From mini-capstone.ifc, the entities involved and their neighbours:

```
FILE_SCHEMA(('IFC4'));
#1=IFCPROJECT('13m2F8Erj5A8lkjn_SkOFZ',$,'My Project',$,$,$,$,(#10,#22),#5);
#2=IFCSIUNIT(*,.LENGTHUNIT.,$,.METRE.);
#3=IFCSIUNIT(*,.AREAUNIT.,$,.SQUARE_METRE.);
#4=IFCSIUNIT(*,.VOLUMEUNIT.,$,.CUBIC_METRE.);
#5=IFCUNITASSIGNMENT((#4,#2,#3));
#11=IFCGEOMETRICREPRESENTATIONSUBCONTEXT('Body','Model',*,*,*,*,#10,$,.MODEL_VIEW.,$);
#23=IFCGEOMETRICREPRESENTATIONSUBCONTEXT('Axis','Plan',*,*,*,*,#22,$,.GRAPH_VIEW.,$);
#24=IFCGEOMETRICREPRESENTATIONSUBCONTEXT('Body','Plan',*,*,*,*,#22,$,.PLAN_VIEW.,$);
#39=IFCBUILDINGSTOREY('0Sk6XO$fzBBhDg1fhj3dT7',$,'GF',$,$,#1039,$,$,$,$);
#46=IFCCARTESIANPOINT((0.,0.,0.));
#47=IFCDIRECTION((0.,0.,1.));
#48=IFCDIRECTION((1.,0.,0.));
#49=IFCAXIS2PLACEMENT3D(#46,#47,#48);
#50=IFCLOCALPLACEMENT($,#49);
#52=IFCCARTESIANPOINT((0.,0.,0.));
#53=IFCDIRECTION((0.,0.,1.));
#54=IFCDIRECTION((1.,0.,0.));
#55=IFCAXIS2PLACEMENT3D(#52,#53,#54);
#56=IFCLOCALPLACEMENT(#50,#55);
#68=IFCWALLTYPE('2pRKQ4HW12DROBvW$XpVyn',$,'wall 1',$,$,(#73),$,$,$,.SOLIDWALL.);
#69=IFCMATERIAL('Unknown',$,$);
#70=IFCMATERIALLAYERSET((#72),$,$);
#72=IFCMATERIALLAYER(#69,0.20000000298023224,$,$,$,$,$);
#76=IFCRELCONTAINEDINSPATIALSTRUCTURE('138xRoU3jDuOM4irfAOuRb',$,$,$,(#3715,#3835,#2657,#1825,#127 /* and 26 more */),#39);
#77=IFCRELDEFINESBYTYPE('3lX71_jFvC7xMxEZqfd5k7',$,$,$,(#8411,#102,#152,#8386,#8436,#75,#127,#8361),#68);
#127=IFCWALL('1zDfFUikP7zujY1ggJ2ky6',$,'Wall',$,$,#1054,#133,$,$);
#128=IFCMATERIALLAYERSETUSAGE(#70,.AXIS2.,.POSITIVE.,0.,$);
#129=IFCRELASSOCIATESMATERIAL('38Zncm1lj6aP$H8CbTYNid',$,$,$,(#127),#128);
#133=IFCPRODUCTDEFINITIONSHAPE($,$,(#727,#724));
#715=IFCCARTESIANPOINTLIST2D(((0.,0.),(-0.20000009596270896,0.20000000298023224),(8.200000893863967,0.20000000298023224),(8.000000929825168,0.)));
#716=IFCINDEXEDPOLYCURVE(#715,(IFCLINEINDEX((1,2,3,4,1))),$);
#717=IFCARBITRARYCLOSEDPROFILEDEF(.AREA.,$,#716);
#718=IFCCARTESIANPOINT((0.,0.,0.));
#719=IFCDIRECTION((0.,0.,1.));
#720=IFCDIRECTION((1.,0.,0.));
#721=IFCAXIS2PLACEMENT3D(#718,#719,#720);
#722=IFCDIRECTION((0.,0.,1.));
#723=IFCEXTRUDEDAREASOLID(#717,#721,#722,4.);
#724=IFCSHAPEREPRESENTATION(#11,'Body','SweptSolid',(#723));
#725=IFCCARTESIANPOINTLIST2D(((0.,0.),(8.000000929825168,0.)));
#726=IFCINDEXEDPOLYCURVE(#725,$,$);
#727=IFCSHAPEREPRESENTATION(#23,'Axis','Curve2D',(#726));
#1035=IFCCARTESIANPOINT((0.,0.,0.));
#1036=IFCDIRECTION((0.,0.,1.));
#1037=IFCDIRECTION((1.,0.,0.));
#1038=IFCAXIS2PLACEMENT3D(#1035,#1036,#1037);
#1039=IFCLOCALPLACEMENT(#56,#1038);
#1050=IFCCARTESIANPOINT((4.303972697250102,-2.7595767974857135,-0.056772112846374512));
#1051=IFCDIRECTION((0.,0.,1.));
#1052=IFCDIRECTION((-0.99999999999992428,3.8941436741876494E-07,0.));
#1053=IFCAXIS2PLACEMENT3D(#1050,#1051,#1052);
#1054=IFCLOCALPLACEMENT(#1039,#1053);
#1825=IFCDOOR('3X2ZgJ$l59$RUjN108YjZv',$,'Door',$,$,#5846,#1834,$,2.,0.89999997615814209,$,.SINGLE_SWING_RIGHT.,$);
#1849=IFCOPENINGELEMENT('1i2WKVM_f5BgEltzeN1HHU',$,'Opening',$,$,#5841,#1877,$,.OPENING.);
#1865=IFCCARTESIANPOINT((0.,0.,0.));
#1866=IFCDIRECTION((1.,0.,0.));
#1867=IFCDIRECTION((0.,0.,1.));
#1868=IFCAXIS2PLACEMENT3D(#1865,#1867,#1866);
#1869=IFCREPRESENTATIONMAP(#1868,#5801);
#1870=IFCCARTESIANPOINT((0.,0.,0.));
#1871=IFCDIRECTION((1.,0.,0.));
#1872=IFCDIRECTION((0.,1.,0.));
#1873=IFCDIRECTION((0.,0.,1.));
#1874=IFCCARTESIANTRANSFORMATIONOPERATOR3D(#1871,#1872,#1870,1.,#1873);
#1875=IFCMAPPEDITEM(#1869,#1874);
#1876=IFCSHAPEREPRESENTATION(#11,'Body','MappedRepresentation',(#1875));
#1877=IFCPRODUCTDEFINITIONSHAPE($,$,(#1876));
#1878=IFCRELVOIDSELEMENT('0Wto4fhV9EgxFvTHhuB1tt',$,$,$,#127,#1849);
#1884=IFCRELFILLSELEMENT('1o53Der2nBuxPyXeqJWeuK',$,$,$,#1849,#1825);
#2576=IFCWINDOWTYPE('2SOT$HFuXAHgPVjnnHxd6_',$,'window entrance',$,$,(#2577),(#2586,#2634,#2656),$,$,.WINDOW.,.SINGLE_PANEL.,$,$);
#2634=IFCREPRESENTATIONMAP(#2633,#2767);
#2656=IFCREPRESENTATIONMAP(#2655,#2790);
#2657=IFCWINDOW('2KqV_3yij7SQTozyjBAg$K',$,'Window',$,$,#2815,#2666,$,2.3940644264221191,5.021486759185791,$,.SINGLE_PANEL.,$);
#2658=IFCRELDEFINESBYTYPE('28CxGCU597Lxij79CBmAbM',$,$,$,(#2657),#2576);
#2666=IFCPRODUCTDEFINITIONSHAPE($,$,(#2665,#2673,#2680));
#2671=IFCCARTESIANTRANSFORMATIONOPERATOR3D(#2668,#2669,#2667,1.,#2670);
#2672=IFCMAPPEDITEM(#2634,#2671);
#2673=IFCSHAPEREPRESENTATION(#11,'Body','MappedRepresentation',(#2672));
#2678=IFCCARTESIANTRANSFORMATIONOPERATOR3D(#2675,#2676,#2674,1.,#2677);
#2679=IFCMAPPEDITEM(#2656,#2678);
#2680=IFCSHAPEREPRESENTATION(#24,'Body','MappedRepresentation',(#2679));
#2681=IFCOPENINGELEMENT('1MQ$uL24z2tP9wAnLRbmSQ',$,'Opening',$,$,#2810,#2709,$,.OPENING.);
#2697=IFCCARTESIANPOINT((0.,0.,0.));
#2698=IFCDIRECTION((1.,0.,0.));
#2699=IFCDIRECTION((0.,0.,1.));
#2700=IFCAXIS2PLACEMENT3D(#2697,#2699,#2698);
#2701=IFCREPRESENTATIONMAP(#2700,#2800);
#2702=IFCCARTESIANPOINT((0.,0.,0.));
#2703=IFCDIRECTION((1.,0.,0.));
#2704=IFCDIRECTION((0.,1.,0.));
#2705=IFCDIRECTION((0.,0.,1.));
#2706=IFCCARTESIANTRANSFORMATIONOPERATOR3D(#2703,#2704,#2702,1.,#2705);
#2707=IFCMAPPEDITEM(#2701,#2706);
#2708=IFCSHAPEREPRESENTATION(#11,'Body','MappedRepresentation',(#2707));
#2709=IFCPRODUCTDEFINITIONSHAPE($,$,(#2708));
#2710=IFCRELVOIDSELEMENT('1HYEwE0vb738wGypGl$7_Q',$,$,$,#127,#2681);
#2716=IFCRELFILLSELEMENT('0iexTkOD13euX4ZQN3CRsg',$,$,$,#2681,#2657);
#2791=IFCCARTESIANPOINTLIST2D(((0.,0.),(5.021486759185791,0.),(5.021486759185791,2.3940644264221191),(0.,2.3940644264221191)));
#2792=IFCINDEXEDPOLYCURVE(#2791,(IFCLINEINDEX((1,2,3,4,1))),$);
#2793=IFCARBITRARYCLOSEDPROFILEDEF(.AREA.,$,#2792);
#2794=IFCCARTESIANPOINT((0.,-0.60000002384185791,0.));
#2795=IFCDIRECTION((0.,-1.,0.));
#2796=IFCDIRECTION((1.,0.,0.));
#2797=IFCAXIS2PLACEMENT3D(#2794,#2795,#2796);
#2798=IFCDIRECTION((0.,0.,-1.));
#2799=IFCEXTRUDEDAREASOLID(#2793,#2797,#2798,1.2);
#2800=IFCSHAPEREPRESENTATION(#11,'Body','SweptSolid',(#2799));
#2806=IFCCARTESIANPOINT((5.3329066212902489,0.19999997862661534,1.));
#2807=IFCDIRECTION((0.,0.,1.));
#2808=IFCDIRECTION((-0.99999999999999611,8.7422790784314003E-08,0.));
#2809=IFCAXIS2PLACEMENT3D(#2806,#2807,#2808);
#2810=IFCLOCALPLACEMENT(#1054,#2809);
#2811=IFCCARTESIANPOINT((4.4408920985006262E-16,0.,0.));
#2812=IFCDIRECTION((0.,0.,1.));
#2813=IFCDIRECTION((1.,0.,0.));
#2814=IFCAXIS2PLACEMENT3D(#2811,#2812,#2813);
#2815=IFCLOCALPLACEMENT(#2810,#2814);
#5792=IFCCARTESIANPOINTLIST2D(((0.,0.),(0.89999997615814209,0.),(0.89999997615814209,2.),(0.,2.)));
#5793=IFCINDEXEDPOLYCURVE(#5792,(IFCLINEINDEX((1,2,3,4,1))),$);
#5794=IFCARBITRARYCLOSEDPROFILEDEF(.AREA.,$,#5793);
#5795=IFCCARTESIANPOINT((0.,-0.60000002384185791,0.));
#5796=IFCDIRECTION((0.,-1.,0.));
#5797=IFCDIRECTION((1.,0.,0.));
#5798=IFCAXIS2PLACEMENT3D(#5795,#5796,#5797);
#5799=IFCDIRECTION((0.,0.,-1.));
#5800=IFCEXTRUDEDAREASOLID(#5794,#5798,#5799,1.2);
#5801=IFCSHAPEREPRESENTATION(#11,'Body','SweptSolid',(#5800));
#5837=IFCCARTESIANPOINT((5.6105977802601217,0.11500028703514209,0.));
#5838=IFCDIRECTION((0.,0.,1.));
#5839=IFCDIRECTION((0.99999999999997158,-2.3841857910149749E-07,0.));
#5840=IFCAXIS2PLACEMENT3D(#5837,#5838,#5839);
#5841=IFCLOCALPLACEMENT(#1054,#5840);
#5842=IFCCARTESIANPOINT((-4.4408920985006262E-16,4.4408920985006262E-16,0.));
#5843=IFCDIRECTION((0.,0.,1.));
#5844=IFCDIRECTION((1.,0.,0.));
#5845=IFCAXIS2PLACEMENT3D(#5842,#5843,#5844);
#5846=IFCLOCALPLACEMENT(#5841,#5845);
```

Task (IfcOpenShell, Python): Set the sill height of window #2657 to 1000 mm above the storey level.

```python
import numpy as np
import ifcopenshell
import ifcopenshell.api.geometry
import ifcopenshell.geom
import ifcopenshell.util.element
import ifcopenshell.util.placement
import ifcopenshell.util.shape
import ifcopenshell.util.unit

model = ifcopenshell.open("mini-capstone.ifc")
unit_scale = ifcopenshell.util.unit.calculate_unit_scale(model)

window = model.by_id(2657)
opening = window.FillsVoids[0].RelatingOpeningElement
storey = ifcopenshell.util.element.get_container(window, ifc_class="IfcBuildingStorey")
level = ifcopenshell.util.placement.get_local_placement(storey.ObjectPlacement)[2, 3]

# The opening's origin need not be at the sill, so measure its lowest point.
shape = ifcopenshell.geom.create_shape(ifcopenshell.geom.settings(), opening)
bottom = ifcopenshell.util.shape.get_shape_bottom_elevation(shape, shape.geometry) / unit_scale
dz = level + 1 / unit_scale - bottom

shift = np.array([0.0, 0.0, dz])
# The window is placed relative to its opening, so it follows when the opening moves.
matrix = ifcopenshell.util.placement.get_local_placement(opening.ObjectPlacement)
matrix[:3, 3] += shift
ifcopenshell.api.geometry.edit_object_placement(
    model, product=opening, matrix=matrix, is_si=False, should_transform_children=True
)

print(f"moved by {dz * unit_scale:+.3f} m")

model.write("mini-capstone_v2.ifc")
```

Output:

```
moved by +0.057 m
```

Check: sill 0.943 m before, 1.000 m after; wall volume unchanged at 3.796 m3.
